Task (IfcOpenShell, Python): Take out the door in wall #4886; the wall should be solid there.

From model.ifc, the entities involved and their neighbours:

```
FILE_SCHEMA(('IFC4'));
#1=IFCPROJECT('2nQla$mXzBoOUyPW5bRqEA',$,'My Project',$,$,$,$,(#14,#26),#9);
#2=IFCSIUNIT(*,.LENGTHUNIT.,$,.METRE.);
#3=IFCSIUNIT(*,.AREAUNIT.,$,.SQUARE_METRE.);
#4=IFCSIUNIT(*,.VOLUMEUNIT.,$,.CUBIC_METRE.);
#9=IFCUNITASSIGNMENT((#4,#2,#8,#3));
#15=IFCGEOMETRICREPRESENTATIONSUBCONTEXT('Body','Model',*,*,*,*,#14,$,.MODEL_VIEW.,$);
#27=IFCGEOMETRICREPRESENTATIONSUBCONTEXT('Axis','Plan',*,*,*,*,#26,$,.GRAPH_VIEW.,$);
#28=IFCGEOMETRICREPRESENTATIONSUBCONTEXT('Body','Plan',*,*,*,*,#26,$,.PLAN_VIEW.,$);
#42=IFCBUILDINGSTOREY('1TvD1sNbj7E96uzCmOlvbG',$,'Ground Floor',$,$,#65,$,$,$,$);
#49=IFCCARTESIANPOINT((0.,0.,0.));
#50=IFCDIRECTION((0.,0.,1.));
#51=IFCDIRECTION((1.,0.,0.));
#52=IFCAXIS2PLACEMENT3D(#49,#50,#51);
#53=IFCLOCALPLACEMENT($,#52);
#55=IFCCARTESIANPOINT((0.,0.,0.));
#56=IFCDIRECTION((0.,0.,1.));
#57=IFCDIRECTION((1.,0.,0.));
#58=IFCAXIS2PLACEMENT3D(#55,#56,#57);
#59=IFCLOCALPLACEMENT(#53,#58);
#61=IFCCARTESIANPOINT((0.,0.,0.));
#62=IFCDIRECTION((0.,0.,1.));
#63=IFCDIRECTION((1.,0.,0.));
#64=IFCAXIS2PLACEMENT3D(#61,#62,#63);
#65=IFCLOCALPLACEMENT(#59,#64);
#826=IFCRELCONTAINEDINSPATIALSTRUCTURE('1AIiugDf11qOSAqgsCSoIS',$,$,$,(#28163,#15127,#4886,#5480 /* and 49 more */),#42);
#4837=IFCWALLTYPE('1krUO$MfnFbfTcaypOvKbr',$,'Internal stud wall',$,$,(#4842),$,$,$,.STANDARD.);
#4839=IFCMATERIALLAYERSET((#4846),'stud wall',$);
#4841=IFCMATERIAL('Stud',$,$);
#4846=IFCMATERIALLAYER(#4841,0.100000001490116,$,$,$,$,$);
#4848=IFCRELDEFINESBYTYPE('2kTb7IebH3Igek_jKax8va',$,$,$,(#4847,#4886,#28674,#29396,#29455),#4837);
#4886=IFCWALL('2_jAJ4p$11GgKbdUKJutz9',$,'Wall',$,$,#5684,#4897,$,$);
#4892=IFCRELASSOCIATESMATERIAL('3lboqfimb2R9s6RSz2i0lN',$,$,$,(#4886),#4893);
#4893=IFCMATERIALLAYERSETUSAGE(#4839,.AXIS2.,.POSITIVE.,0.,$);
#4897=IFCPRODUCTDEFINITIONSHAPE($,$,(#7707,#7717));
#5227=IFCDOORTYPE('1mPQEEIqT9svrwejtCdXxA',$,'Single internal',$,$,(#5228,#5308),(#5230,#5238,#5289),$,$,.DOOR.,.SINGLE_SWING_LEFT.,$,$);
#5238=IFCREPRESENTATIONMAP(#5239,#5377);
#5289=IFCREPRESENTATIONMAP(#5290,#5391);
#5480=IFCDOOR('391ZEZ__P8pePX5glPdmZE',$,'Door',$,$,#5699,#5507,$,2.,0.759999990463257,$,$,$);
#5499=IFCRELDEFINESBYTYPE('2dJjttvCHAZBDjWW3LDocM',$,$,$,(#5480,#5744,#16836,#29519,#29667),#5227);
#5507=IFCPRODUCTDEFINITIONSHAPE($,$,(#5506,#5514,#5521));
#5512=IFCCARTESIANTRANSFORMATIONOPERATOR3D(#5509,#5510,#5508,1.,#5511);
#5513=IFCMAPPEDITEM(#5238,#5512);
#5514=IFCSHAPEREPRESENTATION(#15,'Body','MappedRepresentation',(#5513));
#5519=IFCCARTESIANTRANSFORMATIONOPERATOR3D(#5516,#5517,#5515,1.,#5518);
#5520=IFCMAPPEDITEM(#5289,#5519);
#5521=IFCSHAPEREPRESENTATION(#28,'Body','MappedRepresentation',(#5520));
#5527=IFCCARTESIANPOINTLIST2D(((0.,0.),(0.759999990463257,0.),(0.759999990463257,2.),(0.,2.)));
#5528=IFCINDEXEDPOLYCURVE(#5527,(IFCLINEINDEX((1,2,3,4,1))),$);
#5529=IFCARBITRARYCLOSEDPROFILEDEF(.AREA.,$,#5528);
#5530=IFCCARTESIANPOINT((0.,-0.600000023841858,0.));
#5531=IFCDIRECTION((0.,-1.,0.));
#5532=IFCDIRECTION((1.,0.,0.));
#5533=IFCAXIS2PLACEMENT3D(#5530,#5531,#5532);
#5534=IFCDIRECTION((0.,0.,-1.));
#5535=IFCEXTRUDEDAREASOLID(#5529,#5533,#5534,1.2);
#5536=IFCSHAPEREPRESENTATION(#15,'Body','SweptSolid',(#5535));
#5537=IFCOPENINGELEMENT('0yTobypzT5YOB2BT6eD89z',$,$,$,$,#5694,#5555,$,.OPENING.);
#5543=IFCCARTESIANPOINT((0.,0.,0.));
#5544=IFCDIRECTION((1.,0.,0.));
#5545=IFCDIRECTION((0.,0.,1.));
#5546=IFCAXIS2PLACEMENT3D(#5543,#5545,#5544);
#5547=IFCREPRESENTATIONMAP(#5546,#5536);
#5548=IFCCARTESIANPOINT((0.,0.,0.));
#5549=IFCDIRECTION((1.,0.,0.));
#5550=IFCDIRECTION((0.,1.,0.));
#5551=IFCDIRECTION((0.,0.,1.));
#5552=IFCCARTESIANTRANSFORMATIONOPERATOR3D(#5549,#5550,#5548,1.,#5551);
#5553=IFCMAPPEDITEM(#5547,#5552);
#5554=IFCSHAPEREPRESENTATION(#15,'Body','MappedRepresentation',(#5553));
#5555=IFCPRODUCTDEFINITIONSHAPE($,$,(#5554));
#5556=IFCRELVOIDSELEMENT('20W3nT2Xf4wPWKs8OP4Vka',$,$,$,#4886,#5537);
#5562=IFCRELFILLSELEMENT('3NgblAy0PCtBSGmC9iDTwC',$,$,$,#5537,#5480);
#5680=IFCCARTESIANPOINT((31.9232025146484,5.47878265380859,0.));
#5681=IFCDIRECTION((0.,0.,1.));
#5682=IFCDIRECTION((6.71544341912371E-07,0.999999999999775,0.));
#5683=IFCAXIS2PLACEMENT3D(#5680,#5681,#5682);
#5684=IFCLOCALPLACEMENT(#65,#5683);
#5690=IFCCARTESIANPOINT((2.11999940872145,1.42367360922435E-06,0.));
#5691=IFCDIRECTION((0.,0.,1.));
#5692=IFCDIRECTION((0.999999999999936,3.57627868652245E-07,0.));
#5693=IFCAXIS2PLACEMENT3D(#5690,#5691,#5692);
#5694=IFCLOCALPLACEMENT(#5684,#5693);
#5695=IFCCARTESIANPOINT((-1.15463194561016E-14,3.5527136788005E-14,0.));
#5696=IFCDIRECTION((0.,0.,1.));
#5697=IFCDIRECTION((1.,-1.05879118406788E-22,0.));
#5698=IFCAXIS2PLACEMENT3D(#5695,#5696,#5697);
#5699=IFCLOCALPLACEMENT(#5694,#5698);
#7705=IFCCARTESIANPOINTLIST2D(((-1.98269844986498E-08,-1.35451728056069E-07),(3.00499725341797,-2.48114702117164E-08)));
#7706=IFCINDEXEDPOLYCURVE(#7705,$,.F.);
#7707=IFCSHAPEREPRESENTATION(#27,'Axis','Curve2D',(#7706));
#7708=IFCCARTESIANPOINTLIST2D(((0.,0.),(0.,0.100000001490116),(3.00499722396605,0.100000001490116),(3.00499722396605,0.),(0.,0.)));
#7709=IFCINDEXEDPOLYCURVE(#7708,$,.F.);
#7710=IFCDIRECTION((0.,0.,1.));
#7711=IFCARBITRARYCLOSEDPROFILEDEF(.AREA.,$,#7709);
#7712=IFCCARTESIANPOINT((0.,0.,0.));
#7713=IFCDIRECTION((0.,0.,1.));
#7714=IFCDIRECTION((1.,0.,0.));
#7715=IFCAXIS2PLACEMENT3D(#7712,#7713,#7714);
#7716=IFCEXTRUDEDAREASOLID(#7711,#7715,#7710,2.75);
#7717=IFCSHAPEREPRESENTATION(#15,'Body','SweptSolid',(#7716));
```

```python
import ifcopenshell
import ifcopenshell.api.feature
import ifcopenshell.api.root
import ifcopenshell.geom
import ifcopenshell.util.shape

model = ifcopenshell.open("model.ifc")
settings = ifcopenshell.geom.settings()


def volume(element):
    """Net volume in cubic metres, openings subtracted."""
    shape = ifcopenshell.geom.create_shape(settings, element)
    return ifcopenshell.util.shape.get_volume(shape.geometry)


door = model.by_guid("391ZEZ__P8pePX5glPdmZE")
opening = door.FillsVoids[0].RelatingOpeningElement
wall = opening.VoidsElements[0].RelatingBuildingElement
before = volume(wall)

ifcopenshell.api.root.remove_product(model, product=door)
ifcopenshell.api.feature.remove_feature(model, feature=opening)

after = volume(wall)

print(f"wall volume {before:.3f} -> {after:.3f} m3")

model.write("model_rev.ifc")
```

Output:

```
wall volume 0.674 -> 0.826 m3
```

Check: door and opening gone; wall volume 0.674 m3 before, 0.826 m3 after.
